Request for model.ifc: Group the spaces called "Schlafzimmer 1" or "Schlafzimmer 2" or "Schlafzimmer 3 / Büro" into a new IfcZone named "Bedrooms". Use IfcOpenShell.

First a look at what the model holds.

```python
import ifcopenshell

model = ifcopenshell.open("model.ifc")
print(model.schema)
seen = {}
for space in model.by_type("IfcSpace"):
    seen[space.LongName] = seen.get(space.LongName, 0) + 1
for name, count in sorted(seen.items(), key=str):
    print(count, "x", name)
print("zones:", [z.Name for z in model.by_type("IfcZone")][:20])
```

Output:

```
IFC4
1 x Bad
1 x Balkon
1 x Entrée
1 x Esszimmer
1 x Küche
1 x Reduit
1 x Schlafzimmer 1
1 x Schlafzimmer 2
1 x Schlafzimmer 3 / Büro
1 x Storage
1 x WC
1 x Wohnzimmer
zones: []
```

```python
import ifcopenshell
import ifcopenshell.api.group
import ifcopenshell.api.root

model = ifcopenshell.open("model.ifc")

names = {"Schlafzimmer 1", "Schlafzimmer 2", "Schlafzimmer 3 / Büro"}
spaces = [s for s in model.by_type("IfcSpace") if s.LongName in names]

zone = ifcopenshell.api.root.create_entity(model, ifc_class="IfcZone", name="Bedrooms")
ifcopenshell.api.group.assign_group(model, products=spaces, group=zone)
print(len(spaces), "spaces in", zone.Name)

model.write("model_edited.ifc")
```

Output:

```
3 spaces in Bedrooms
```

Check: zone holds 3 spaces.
